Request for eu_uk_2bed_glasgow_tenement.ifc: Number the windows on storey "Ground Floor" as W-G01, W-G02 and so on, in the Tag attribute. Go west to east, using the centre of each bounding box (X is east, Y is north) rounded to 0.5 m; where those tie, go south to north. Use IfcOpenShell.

First a look at what the model holds.

```python
import ifcopenshell
import ifcopenshell.util.element
import ifcopenshell.util.placement

model = ifcopenshell.open("eu_uk_2bed_glasgow_tenement.ifc")
print(model.schema)
storey = next(s for s in model.by_type("IfcBuildingStorey") if s.Name == "Ground Floor")
windows = [e for e in ifcopenshell.util.element.get_decomposition(storey) if e.is_a("IfcWindow")]
for e in sorted(windows, key=lambda e: e.id()):
    origin = ifcopenshell.util.placement.get_local_placement(e.ObjectPlacement)[:3, 3]
    print(e.id(), e.Tag, e.Name, origin.round(2) + 0.0, sep=" | ")
```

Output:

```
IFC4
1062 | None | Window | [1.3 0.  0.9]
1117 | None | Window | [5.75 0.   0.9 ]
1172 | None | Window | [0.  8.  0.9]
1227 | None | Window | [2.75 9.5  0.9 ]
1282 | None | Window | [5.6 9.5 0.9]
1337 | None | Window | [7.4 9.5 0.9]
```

```python
import ifcopenshell
import ifcopenshell.geom
import ifcopenshell.util.element
import ifcopenshell.util.shape

model = ifcopenshell.open("eu_uk_2bed_glasgow_tenement.ifc")
settings = ifcopenshell.geom.settings()
settings.set("use-world-coords", True)


def centre(element):
    shape = ifcopenshell.geom.create_shape(settings, element)
    return ifcopenshell.util.shape.get_bbox_centroid(shape.geometry)


storey = next(s for s in model.by_type("IfcBuildingStorey") if s.Name == "Ground Floor")
windows = [e for e in ifcopenshell.util.element.get_decomposition(storey) if e.is_a("IfcWindow")]

# Insertion points can sit at a corner or the storey origin, so sort by the geometry (in metres).
centres = {e: centre(e) for e in windows}
windows.sort(key=lambda e: (round(centres[e][0] / 0.5), centres[e][1]))

for i, e in enumerate(windows, start=1):
    number = f"W-G{i:02d}"
    e.Tag = number
    print(e.id(), number)

model.write("eu_uk_2bed_glasgow_tenement_edited.ifc")
```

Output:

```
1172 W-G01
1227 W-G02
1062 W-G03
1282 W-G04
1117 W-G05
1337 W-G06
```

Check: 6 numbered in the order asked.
